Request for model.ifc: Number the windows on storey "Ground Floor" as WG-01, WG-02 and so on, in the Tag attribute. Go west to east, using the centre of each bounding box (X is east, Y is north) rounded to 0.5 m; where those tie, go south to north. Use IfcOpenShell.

First a look at what the model holds.

```python
import ifcopenshell
import ifcopenshell.util.element
import ifcopenshell.util.placement

model = ifcopenshell.open("model.ifc")
print(model.schema)
storey = next(s for s in model.by_type("IfcBuildingStorey") if s.Name == "Ground Floor")
windows = [e for e in ifcopenshell.util.element.get_decomposition(storey) if e.is_a("IfcWindow")]
for e in sorted(windows, key=lambda e: e.id()):
    origin = ifcopenshell.util.placement.get_local_placement(e.ObjectPlacement)[:3, 3]
    print(e.id(), e.Tag, e.Name, origin.round(2) + 0.0, sep=" | ")
```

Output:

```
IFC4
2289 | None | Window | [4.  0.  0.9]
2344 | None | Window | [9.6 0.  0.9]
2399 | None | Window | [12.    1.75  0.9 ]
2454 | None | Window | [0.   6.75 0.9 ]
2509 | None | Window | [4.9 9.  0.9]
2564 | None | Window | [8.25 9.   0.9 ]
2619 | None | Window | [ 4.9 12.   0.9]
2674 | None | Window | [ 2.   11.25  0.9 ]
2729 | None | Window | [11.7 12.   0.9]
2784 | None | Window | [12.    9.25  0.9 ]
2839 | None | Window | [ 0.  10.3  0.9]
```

```python
import ifcopenshell
import ifcopenshell.geom
import ifcopenshell.util.element
import ifcopenshell.util.shape

model = ifcopenshell.open("model.ifc")
settings = ifcopenshell.geom.settings()
settings.set("use-world-coords", True)


def centre(element):
    shape = ifcopenshell.geom.create_shape(settings, element)
    return ifcopenshell.util.shape.get_bbox_centroid(shape.geometry)


storey = next(s for s in model.by_type("IfcBuildingStorey") if s.Name == "Ground Floor")
windows = [e for e in ifcopenshell.util.element.get_decomposition(storey) if e.is_a("IfcWindow")]

# Insertion points can sit at a corner or the storey origin, so sort by the geometry (in metres).
centres = {e: centre(e) for e in windows}
windows.sort(key=lambda e: (round(centres[e][0] / 0.5), centres[e][1]))

for i, e in enumerate(windows, start=1):
    number = f"WG-{i:02d}"
    e.Tag = number
    print(e.id(), number)

model.write("model_rev.ifc")
```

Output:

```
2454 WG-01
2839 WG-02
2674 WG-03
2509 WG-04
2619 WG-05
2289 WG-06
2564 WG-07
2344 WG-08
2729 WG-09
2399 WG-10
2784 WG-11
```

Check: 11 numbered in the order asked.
